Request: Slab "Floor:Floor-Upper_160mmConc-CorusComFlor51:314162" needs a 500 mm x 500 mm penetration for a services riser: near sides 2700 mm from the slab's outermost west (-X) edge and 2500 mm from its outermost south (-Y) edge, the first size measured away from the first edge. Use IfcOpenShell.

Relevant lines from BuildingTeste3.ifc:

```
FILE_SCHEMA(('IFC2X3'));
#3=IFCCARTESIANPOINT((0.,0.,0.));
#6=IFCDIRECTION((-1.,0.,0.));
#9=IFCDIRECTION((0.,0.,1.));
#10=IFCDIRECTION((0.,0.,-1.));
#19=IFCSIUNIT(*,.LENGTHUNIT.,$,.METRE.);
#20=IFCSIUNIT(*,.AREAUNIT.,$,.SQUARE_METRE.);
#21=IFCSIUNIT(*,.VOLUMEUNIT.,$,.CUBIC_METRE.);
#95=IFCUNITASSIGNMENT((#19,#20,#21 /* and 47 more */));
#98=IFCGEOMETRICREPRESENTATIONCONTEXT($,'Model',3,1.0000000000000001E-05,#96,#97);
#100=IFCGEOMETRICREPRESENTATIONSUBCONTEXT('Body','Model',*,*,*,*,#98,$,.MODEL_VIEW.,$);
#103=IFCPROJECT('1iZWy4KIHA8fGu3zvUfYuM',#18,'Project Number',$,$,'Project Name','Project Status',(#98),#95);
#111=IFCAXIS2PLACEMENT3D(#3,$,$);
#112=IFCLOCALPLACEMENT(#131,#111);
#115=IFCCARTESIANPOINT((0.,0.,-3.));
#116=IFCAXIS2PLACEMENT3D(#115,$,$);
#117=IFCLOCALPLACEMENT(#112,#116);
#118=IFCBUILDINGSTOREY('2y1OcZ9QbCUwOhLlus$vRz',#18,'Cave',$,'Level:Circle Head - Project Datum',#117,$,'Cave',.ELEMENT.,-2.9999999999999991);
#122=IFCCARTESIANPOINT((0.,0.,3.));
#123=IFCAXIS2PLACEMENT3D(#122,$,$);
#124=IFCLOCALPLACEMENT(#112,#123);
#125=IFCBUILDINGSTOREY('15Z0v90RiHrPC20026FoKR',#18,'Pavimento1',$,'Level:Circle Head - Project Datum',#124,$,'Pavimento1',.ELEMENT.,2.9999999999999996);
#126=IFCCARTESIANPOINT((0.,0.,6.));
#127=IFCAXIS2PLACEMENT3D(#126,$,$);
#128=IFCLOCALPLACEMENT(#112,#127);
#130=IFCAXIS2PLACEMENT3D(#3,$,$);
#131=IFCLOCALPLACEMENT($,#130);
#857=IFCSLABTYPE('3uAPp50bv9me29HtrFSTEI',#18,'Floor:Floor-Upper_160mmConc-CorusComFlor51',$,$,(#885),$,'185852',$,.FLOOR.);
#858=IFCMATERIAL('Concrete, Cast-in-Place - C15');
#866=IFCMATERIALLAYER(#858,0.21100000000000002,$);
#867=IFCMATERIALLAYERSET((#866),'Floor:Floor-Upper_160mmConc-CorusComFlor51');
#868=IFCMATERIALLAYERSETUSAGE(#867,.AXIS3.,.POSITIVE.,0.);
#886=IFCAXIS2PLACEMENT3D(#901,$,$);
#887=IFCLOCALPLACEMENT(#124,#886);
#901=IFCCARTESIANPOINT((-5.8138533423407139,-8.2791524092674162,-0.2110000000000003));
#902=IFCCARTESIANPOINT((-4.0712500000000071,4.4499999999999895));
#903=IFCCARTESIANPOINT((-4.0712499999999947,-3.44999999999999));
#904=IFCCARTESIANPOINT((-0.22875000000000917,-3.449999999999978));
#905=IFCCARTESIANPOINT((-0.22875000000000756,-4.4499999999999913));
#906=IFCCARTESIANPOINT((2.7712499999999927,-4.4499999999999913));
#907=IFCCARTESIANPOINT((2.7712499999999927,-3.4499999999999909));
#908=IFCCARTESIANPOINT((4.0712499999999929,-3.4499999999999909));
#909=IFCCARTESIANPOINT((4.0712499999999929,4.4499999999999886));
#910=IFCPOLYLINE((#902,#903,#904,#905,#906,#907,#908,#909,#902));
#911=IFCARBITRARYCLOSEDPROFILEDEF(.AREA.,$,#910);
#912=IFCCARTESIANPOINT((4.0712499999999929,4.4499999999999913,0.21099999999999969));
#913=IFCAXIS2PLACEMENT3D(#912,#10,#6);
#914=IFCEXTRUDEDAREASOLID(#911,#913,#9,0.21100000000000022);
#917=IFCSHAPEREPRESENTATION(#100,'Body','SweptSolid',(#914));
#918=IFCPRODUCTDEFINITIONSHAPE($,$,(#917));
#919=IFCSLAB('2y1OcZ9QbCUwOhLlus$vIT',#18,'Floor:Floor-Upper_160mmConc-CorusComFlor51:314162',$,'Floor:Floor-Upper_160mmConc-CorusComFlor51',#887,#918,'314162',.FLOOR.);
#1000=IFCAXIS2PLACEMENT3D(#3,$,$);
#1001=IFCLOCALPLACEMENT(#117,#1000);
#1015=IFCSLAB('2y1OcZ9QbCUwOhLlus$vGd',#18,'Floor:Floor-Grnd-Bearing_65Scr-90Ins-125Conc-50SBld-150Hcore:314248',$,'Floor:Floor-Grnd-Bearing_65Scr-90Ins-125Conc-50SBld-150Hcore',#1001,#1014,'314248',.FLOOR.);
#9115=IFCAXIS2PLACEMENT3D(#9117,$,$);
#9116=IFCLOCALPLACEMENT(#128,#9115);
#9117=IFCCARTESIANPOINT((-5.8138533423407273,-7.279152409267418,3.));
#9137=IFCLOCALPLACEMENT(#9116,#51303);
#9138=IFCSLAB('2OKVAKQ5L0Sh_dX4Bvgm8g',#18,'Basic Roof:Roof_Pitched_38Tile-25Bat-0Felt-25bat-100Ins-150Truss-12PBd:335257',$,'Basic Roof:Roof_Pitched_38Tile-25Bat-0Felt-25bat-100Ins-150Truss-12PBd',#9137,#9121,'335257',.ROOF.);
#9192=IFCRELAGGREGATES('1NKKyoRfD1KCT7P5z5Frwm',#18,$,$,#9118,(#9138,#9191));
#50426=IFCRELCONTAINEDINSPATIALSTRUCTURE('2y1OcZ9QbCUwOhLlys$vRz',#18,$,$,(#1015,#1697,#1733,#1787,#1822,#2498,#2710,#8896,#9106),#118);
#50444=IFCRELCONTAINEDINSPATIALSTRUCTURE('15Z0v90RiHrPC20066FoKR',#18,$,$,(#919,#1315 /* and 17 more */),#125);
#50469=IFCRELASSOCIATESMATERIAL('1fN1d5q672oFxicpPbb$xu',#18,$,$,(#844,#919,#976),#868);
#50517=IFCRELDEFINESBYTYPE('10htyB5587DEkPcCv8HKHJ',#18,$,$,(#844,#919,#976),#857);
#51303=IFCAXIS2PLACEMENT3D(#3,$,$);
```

```python
import numpy as np
import ifcopenshell
import ifcopenshell.api.feature
import ifcopenshell.api.geometry
import ifcopenshell.api.root
import ifcopenshell.geom
import ifcopenshell.util.placement
import ifcopenshell.util.representation
import ifcopenshell.util.shape
import ifcopenshell.util.unit

model = ifcopenshell.open("BuildingTeste3.ifc")
unit_scale = ifcopenshell.util.unit.calculate_unit_scale(model)
settings = ifcopenshell.geom.settings()


def volume(element):
    """Net volume in cubic metres, openings subtracted."""
    shape = ifcopenshell.geom.create_shape(settings, element)
    return ifcopenshell.util.shape.get_volume(shape.geometry)


slab = model.by_guid("2y1OcZ9QbCUwOhLlus$vIT")
before = volume(slab)

# Extent in the slab's own axes, in metres. The edges named are its -X and -Y sides.
slab_shape = ifcopenshell.geom.create_shape(settings, slab)
vertices = ifcopenshell.util.shape.get_vertices(slab_shape.geometry)
x_min, y_min, bottom = vertices.min(axis=0)
top = vertices[:, 2].max()

opening = ifcopenshell.api.root.create_entity(model, ifc_class="IfcOpeningElement", name="Services riser opening")
context = ifcopenshell.util.representation.get_context(model, "Model", "Body", "MODEL_VIEW")
width, depth = 0.5, 0.5
outline = [(0.0, 0.0), (width, 0.0), (width, depth), (0.0, depth), (0.0, 0.0)]
# Overshoot both faces by 50 mm so the cut is clean.
shape = ifcopenshell.api.geometry.add_slab_representation(
    model, context=context, depth=top - bottom + 0.1, polyline=outline
)
ifcopenshell.api.geometry.assign_representation(model, product=opening, representation=shape)

matrix = ifcopenshell.util.placement.get_local_placement(slab.ObjectPlacement)
matrix[:, 3] = matrix @ np.append(np.array([x_min + 2.7, y_min + 2.5, bottom - 0.05]) / unit_scale, 1.0)
ifcopenshell.api.geometry.edit_object_placement(model, product=opening, matrix=matrix, is_si=False)
ifcopenshell.api.feature.add_feature(model, feature=opening, element=slab)

after = volume(slab)

print(f"slab volume {before:.3f} -> {after:.3f} m3")

model.write("BuildingTeste3_v2.ifc")
```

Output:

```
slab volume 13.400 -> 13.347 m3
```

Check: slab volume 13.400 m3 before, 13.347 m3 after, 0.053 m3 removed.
